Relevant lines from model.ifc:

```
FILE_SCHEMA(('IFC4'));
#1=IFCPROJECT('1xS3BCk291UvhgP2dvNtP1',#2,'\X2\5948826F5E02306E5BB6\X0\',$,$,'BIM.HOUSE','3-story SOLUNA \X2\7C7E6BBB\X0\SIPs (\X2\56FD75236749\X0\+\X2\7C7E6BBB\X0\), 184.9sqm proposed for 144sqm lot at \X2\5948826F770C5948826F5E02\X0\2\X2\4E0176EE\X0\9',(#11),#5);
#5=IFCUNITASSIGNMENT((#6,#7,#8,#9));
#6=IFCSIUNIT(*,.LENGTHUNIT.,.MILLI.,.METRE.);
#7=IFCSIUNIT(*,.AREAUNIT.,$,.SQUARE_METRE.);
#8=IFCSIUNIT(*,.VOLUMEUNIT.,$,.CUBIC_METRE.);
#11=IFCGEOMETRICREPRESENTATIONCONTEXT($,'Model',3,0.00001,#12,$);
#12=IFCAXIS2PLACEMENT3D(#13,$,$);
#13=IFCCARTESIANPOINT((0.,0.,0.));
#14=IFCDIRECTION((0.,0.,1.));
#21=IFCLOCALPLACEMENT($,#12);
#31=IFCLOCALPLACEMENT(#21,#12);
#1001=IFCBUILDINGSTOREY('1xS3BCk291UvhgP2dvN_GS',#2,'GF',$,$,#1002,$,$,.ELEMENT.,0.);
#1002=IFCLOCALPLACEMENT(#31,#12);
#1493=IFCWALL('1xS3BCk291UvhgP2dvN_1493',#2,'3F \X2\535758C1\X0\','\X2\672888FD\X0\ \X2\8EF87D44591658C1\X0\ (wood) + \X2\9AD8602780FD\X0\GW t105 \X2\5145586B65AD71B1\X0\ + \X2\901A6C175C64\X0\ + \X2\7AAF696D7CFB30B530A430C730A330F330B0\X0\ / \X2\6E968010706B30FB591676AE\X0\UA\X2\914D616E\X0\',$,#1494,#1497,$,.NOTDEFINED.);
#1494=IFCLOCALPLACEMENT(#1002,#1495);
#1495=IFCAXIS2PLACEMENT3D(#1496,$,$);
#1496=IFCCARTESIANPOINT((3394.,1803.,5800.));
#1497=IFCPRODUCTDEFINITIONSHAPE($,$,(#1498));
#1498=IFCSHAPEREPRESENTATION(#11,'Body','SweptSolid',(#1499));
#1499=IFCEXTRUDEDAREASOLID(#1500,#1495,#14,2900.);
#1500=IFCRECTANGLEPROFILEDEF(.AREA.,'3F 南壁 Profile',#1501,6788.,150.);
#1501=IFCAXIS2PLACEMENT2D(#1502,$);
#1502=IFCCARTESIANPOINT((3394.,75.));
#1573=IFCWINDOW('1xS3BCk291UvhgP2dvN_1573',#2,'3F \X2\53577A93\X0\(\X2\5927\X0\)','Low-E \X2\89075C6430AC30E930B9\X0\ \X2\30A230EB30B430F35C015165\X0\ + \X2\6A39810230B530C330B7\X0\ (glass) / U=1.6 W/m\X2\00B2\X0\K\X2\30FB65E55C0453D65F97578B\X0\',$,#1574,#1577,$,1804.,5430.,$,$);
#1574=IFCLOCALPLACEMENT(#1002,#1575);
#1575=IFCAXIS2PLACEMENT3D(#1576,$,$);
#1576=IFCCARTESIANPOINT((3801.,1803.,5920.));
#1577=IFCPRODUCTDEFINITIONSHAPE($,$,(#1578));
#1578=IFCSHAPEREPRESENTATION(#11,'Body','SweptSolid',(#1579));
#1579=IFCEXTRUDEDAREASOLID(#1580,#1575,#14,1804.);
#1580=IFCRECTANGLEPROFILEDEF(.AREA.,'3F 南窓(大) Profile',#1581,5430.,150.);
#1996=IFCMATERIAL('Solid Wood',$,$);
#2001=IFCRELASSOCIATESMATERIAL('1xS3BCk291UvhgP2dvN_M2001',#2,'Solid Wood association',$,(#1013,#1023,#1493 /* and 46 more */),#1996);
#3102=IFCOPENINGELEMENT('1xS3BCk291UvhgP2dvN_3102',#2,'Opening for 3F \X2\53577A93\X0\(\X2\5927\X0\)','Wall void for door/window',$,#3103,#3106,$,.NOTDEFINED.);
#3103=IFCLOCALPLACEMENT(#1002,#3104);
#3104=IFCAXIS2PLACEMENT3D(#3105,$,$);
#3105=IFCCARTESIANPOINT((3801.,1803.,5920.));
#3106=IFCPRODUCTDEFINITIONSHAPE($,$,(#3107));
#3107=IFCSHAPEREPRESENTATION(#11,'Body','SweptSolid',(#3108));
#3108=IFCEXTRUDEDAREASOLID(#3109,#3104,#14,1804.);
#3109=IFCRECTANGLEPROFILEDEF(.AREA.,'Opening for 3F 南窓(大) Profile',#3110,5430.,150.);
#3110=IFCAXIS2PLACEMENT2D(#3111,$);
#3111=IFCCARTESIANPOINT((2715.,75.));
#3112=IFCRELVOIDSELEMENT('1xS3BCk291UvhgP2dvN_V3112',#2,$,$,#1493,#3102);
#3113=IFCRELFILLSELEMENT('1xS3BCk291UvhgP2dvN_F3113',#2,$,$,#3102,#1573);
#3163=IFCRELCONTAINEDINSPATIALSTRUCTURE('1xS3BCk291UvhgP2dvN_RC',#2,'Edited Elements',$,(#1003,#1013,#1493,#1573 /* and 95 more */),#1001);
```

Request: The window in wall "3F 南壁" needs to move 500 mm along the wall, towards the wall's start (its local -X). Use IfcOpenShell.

```python
import ifcopenshell
import ifcopenshell.api.geometry
import ifcopenshell.util.placement
import ifcopenshell.util.unit

model = ifcopenshell.open("model.ifc")
unit_scale = ifcopenshell.util.unit.calculate_unit_scale(model)

window = model.by_guid("1xS3BCk291UvhgP2dvN_1573")
opening = window.FillsVoids[0].RelatingOpeningElement
wall = opening.VoidsElements[0].RelatingBuildingElement

wall_matrix = ifcopenshell.util.placement.get_local_placement(wall.ObjectPlacement)
shift = wall_matrix[:3, 0] * -0.5 / unit_scale
before = ifcopenshell.util.placement.get_local_placement(window.ObjectPlacement)[:3, 3].copy()

# The window is not placed relative to its opening, so move both.
for product in (opening, window):
    matrix = ifcopenshell.util.placement.get_local_placement(product.ObjectPlacement)
    matrix[:3, 3] += shift
    ifcopenshell.api.geometry.edit_object_placement(model, product=product, matrix=matrix, is_si=False)

after = ifcopenshell.util.placement.get_local_placement(window.ObjectPlacement)[:3, 3]
print("window moved by", (after - before).round(3) + 0.0)

model.write("model-out.ifc")
```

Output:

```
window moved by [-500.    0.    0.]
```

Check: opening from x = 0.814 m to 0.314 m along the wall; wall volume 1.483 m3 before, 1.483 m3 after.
